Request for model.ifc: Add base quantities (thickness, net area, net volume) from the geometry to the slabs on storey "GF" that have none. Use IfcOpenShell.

First a look at what the model holds.

```python
import ifcopenshell
import ifcopenshell.util.element
import ifcopenshell.util.unit

model = ifcopenshell.open("model.ifc")
print(model.schema)
for unit_type in ("LENGTHUNIT", "AREAUNIT", "VOLUMEUNIT"):
    print(unit_type, ifcopenshell.util.unit.calculate_unit_scale(model, unit_type))
storey = next(s for s in model.by_type("IfcBuildingStorey") if s.Name == "GF")
slabs = [e for e in ifcopenshell.util.element.get_decomposition(storey) if e.is_a("IfcSlab")]
for e in sorted(slabs, key=lambda e: e.id()):
    print(e.id(), e.is_a(), e.Name, list(ifcopenshell.util.element.get_psets(e, qtos_only=True)), sep=" | ")
```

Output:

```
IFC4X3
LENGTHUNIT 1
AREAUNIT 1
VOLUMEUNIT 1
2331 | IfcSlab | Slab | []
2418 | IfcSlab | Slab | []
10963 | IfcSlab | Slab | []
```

```python
import ifcopenshell
import ifcopenshell.api.pset
import ifcopenshell.geom
import ifcopenshell.util.element
import ifcopenshell.util.shape
import ifcopenshell.util.unit

model = ifcopenshell.open("model.ifc")
unit_scale = ifcopenshell.util.unit.calculate_unit_scale(model)
area_scale = ifcopenshell.util.unit.calculate_unit_scale(model, "AREAUNIT")
volume_scale = ifcopenshell.util.unit.calculate_unit_scale(model, "VOLUMEUNIT")
settings = ifcopenshell.geom.settings()

storey = next(s for s in model.by_type("IfcBuildingStorey") if s.Name == "GF")
slabs = [e for e in ifcopenshell.util.element.get_decomposition(storey) if e.is_a("IfcSlab")]

for e in sorted(slabs, key=lambda e: e.id()):
    if ifcopenshell.util.element.get_psets(e, qtos_only=True, should_inherit=False):
        continue
    # Geometry comes back in metres, in the element's own axes.
    shape = ifcopenshell.geom.create_shape(settings, e)
    values = {
        "Width": ifcopenshell.util.shape.get_z(shape.geometry) / unit_scale,
        "NetArea": ifcopenshell.util.shape.get_footprint_area(shape.geometry) / area_scale,
        "NetVolume": ifcopenshell.util.shape.get_volume(shape.geometry) / volume_scale,
    }
    qto = ifcopenshell.api.pset.add_qto(model, product=e, name="Qto_SlabBaseQuantities")
    ifcopenshell.api.pset.edit_qto(model, qto=qto, properties=values)
    print(e.id(), {k: round(v, 3) for k, v in values.items()})

model.write("model_updated.ifc")
```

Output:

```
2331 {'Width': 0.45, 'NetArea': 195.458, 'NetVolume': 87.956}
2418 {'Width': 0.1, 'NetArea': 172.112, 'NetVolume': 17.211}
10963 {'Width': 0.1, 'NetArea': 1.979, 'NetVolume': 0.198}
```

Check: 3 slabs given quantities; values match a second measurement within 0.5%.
